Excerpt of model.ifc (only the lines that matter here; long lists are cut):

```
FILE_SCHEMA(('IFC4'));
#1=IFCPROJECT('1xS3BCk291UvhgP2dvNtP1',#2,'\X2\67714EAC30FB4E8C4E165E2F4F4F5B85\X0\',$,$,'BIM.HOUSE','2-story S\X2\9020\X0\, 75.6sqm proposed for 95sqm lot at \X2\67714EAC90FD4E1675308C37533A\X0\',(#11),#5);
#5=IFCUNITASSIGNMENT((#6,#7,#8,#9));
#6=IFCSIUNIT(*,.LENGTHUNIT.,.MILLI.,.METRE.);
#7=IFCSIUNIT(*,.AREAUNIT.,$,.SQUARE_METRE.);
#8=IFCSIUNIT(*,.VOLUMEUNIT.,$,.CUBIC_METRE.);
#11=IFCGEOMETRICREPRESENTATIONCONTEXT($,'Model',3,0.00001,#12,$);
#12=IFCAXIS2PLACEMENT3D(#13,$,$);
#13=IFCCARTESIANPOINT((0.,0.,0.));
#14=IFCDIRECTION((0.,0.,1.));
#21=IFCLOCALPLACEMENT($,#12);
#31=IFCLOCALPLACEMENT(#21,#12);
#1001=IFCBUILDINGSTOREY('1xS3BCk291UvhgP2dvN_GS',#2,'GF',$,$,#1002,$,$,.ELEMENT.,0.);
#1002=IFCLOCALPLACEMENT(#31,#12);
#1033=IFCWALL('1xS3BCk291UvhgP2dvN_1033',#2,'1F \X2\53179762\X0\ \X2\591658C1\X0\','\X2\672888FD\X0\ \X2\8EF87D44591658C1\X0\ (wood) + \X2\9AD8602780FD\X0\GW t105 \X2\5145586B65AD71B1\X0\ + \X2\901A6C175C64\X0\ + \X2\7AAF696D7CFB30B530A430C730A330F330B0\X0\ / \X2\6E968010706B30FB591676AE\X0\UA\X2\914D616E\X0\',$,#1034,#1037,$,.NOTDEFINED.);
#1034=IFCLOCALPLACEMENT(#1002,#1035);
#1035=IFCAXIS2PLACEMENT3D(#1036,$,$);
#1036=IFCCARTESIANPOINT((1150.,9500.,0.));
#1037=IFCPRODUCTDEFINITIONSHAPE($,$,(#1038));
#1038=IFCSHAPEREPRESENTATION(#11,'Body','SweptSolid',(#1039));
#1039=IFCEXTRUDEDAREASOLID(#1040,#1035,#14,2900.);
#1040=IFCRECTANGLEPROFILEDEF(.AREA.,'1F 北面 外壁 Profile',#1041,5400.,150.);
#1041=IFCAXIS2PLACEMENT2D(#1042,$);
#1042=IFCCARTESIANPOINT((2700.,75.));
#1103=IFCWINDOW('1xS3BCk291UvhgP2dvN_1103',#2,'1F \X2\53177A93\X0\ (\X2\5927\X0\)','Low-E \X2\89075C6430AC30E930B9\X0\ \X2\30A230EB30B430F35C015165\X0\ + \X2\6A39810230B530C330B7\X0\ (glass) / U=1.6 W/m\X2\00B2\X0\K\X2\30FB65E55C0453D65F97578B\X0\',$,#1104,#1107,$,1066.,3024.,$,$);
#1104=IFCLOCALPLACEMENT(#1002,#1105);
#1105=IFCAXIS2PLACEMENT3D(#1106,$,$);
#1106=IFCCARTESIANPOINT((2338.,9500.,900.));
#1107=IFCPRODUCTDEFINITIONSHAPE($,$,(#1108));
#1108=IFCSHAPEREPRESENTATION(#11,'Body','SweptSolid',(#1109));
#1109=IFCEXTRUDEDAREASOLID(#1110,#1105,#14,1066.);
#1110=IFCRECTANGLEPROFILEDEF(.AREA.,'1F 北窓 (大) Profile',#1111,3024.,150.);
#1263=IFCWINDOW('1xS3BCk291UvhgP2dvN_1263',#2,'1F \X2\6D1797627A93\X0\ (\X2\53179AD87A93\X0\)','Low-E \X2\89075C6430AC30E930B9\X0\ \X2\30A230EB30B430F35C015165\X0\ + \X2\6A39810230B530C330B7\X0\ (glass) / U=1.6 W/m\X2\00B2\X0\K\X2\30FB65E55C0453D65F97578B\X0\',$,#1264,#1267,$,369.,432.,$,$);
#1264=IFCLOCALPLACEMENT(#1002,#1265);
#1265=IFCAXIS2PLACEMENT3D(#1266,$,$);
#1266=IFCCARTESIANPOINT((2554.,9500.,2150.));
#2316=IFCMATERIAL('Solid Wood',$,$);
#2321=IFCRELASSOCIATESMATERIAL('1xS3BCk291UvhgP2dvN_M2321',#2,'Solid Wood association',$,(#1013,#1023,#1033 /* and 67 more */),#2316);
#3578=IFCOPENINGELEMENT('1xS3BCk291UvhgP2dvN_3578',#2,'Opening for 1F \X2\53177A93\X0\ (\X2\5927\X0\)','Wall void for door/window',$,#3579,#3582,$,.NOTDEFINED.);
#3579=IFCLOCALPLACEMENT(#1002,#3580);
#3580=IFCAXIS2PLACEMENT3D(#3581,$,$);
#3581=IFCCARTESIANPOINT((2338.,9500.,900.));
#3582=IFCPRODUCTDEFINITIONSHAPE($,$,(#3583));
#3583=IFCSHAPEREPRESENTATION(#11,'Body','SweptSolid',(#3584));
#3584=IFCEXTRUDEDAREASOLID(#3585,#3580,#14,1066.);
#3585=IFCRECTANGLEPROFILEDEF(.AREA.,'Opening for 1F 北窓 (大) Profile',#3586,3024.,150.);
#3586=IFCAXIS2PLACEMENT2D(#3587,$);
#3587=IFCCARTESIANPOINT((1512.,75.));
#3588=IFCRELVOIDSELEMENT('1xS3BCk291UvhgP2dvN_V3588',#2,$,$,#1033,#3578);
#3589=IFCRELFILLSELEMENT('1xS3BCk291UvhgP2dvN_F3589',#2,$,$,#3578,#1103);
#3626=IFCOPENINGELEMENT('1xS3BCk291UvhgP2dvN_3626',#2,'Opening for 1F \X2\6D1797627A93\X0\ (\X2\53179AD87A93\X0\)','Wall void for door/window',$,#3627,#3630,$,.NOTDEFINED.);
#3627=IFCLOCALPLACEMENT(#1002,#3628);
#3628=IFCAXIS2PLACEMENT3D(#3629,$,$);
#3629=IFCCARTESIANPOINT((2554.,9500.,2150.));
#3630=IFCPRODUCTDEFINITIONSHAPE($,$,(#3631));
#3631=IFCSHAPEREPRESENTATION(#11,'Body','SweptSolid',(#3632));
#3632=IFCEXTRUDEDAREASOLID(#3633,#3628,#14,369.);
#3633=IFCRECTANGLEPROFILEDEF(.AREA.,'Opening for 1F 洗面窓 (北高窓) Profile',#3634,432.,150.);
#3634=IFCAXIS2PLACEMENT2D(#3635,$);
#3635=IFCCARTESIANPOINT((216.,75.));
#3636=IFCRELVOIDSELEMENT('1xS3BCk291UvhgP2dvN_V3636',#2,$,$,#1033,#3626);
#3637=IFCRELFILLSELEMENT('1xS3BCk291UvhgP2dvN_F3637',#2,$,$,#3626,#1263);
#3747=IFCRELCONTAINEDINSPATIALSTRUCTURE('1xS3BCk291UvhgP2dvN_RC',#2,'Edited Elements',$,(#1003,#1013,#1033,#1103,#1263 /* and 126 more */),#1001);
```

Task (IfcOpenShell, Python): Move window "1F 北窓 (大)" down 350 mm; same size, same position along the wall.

```python
import numpy as np
import ifcopenshell
import ifcopenshell.api.geometry
import ifcopenshell.util.placement
import ifcopenshell.util.unit

model = ifcopenshell.open("model.ifc")
unit_scale = ifcopenshell.util.unit.calculate_unit_scale(model)

window = model.by_guid("1xS3BCk291UvhgP2dvN_1103")
opening = window.FillsVoids[0].RelatingOpeningElement
dz = -0.35 / unit_scale

shift = np.array([0.0, 0.0, dz])
# The window is not placed relative to its opening, so move both.
for product in (opening, window):
    matrix = ifcopenshell.util.placement.get_local_placement(product.ObjectPlacement)
    matrix[:3, 3] += shift
    ifcopenshell.api.geometry.edit_object_placement(model, product=product, matrix=matrix, is_si=False)

print(f"moved by {dz * unit_scale:+.3f} m")

model.write("model_updated.ifc")
```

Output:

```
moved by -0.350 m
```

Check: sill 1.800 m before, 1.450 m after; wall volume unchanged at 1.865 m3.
